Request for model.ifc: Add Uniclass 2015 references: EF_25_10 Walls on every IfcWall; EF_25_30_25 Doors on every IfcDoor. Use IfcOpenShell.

First a look at what the model holds.

```python
import ifcopenshell

model = ifcopenshell.open("model.ifc")
print(model.schema)
print("classifications:", [c.Name for c in model.by_type("IfcClassification")])
for ifc_class in ("IfcDoor", "IfcRoof", "IfcStair", "IfcWall", "IfcWindow"):
    print(ifc_class, len(model.by_type(ifc_class)))
```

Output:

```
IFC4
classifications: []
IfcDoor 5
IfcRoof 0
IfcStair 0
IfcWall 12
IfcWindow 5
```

```python
import ifcopenshell
import ifcopenshell.api.classification

model = ifcopenshell.open("model.ifc")

system = ifcopenshell.api.classification.add_classification(model, classification="Uniclass 2015")

codes = {
    "IfcWall": ("EF_25_10", "Walls"),
    "IfcDoor": ("EF_25_30_25", "Doors"),
}
for ifc_class, (code, name) in codes.items():
    products = model.by_type(ifc_class)
    ifcopenshell.api.classification.add_reference(
        model, products=products, classification=system, identification=code, name=name
    )
    print(code, len(products))

model.write("model_edited.ifc")
```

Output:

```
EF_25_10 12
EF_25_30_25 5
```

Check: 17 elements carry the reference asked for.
